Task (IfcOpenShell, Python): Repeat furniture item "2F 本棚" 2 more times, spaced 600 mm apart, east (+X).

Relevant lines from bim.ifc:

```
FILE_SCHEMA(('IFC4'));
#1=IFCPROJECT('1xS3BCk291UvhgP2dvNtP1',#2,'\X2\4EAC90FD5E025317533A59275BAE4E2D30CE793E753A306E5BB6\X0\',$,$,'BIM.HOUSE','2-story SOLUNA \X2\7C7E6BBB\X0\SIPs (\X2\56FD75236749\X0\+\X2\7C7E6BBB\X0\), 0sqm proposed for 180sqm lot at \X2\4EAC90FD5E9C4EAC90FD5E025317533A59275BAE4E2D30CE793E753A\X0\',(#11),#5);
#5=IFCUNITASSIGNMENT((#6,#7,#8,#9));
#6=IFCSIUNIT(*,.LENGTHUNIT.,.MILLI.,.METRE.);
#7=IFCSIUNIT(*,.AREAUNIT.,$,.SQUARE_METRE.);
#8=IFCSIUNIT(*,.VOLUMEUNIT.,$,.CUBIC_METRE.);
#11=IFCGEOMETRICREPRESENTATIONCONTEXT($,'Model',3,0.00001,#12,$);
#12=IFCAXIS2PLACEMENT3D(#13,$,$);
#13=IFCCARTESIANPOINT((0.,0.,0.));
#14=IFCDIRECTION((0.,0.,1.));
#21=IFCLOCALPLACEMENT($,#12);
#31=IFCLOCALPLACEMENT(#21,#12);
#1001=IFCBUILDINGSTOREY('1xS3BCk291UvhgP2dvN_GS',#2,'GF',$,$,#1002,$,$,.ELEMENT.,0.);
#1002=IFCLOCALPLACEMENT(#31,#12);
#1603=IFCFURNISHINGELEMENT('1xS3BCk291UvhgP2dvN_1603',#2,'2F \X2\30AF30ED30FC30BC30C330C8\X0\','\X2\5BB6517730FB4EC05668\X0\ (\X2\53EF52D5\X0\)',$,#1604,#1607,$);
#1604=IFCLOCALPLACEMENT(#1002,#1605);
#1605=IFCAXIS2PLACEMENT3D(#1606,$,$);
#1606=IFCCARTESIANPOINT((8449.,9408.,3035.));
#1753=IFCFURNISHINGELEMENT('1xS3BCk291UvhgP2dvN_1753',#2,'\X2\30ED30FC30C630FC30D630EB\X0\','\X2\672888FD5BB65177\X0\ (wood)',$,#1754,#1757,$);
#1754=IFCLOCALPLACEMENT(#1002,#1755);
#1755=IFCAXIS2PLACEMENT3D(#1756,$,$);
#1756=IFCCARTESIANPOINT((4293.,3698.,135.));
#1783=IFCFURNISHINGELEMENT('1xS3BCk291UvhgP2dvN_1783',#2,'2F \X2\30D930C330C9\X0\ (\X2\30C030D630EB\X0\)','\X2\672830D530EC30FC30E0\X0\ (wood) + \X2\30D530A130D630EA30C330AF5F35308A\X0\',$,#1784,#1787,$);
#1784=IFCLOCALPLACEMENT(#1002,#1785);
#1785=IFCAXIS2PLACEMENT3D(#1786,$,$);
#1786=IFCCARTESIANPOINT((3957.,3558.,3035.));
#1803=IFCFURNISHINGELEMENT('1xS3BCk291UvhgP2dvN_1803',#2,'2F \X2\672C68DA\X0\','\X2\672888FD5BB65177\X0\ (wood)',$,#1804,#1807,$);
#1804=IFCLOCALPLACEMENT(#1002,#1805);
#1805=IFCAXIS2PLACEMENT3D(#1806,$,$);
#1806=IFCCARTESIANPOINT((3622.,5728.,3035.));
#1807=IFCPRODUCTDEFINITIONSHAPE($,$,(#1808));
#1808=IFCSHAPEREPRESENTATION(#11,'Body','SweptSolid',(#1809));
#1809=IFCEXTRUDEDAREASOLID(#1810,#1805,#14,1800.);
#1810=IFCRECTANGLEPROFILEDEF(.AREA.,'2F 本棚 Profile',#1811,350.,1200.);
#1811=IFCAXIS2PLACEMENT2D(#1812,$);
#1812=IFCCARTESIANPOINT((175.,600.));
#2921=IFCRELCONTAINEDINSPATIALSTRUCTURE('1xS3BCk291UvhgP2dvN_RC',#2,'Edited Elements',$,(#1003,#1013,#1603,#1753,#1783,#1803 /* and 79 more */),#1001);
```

```python
import numpy as np
import ifcopenshell
import ifcopenshell.api.geometry
import ifcopenshell.api.root
import ifcopenshell.util.element
import ifcopenshell.util.placement

model = ifcopenshell.open("bim.ifc")


def reuse_history(source, copy):
    """copy_class also copies each property set's owner history, people and application; keep the originals."""
    for rel in copy.IsDefinedBy:
        if rel.is_a("IfcRelDefinesByProperties") and (history := rel.RelatingPropertyDefinition.OwnerHistory):
            rel.RelatingPropertyDefinition.OwnerHistory = source.OwnerHistory
            ifcopenshell.util.element.remove_deep2(model, history)


source = model.by_guid("1xS3BCk291UvhgP2dvN_1803")
base = ifcopenshell.util.placement.get_local_placement(source.ObjectPlacement)
step = np.array([1.0, 0.0, 0.0]) * 600.0

for i in range(1, 3):
    copy = ifcopenshell.api.root.copy_class(model, product=source)
    copy.Representation = ifcopenshell.util.element.copy_deep(
        model, source.Representation, exclude=["IfcGeometricRepresentationContext", "IfcRepresentationMap"]
    )
    reuse_history(source, copy)
    matrix = base.copy()
    matrix[:3, 3] += i * step
    print("added at", matrix[:3, 3].round(3) + 0.0)
    ifcopenshell.api.geometry.edit_object_placement(model, product=copy, matrix=matrix, is_si=False)

model.write("bim_updated.ifc")
```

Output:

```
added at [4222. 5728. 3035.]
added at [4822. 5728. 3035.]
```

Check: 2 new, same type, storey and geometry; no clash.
